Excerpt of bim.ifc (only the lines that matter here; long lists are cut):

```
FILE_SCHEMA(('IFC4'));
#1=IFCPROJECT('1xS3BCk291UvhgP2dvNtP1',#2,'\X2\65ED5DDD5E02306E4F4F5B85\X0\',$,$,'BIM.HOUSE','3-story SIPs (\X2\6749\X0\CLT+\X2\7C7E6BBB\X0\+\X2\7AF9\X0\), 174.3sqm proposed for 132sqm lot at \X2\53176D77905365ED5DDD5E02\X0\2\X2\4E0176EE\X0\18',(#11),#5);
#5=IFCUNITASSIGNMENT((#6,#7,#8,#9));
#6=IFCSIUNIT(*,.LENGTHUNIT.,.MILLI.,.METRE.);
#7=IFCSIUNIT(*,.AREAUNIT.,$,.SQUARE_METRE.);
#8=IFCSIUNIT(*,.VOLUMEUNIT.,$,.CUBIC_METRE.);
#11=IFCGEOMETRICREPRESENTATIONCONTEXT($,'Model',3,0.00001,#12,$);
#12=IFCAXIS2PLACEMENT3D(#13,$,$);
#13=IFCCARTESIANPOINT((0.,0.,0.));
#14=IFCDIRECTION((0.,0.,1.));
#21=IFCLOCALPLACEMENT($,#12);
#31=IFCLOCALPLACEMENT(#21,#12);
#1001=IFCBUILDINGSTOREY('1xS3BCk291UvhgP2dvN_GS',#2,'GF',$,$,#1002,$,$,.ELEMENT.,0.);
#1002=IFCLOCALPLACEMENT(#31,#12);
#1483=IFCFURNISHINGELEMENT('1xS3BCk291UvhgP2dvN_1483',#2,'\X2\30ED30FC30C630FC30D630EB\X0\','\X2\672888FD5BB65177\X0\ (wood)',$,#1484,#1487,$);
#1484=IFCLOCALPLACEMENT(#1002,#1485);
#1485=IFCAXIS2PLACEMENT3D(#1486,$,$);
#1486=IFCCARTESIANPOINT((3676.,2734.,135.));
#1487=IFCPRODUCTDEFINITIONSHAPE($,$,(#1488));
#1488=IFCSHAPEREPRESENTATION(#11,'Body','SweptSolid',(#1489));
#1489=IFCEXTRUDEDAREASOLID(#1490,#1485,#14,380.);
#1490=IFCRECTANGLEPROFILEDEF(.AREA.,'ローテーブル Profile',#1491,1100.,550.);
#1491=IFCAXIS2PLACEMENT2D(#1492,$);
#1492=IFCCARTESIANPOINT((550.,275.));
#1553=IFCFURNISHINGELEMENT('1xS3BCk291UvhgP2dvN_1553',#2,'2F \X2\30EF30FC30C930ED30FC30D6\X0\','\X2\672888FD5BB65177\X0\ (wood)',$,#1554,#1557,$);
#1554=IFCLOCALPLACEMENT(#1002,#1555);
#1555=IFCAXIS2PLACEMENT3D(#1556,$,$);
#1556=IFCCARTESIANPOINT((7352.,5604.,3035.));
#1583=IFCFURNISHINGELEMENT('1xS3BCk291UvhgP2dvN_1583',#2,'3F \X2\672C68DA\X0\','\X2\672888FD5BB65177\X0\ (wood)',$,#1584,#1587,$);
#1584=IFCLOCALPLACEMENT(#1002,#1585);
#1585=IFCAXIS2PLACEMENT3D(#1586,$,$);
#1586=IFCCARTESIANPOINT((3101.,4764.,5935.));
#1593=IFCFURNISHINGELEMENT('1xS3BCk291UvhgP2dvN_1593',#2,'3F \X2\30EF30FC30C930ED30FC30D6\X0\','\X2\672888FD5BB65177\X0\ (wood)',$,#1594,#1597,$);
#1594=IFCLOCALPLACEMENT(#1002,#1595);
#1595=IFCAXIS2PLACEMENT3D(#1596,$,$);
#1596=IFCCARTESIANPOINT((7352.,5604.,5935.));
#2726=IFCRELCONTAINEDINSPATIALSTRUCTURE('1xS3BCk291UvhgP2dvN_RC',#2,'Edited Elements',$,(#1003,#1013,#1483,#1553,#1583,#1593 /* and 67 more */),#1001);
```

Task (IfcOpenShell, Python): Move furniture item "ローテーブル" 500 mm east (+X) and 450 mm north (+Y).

```python
import ifcopenshell
import ifcopenshell.api.geometry
import ifcopenshell.util.placement

model = ifcopenshell.open("bim.ifc")

item = model.by_guid("1xS3BCk291UvhgP2dvN_1483")
matrix = ifcopenshell.util.placement.get_local_placement(item.ObjectPlacement)
matrix[0, 3] += 500.0
matrix[1, 3] += 450.0
ifcopenshell.api.geometry.edit_object_placement(model, product=item, matrix=matrix, is_si=False)

print(ifcopenshell.util.placement.get_local_placement(item.ObjectPlacement).round(3) + 0.0)

model.write("bim_v2.ifc")
```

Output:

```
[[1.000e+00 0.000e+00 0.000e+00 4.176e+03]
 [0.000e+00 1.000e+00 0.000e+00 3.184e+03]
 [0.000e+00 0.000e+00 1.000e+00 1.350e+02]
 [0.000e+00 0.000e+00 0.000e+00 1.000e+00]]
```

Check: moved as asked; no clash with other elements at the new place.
